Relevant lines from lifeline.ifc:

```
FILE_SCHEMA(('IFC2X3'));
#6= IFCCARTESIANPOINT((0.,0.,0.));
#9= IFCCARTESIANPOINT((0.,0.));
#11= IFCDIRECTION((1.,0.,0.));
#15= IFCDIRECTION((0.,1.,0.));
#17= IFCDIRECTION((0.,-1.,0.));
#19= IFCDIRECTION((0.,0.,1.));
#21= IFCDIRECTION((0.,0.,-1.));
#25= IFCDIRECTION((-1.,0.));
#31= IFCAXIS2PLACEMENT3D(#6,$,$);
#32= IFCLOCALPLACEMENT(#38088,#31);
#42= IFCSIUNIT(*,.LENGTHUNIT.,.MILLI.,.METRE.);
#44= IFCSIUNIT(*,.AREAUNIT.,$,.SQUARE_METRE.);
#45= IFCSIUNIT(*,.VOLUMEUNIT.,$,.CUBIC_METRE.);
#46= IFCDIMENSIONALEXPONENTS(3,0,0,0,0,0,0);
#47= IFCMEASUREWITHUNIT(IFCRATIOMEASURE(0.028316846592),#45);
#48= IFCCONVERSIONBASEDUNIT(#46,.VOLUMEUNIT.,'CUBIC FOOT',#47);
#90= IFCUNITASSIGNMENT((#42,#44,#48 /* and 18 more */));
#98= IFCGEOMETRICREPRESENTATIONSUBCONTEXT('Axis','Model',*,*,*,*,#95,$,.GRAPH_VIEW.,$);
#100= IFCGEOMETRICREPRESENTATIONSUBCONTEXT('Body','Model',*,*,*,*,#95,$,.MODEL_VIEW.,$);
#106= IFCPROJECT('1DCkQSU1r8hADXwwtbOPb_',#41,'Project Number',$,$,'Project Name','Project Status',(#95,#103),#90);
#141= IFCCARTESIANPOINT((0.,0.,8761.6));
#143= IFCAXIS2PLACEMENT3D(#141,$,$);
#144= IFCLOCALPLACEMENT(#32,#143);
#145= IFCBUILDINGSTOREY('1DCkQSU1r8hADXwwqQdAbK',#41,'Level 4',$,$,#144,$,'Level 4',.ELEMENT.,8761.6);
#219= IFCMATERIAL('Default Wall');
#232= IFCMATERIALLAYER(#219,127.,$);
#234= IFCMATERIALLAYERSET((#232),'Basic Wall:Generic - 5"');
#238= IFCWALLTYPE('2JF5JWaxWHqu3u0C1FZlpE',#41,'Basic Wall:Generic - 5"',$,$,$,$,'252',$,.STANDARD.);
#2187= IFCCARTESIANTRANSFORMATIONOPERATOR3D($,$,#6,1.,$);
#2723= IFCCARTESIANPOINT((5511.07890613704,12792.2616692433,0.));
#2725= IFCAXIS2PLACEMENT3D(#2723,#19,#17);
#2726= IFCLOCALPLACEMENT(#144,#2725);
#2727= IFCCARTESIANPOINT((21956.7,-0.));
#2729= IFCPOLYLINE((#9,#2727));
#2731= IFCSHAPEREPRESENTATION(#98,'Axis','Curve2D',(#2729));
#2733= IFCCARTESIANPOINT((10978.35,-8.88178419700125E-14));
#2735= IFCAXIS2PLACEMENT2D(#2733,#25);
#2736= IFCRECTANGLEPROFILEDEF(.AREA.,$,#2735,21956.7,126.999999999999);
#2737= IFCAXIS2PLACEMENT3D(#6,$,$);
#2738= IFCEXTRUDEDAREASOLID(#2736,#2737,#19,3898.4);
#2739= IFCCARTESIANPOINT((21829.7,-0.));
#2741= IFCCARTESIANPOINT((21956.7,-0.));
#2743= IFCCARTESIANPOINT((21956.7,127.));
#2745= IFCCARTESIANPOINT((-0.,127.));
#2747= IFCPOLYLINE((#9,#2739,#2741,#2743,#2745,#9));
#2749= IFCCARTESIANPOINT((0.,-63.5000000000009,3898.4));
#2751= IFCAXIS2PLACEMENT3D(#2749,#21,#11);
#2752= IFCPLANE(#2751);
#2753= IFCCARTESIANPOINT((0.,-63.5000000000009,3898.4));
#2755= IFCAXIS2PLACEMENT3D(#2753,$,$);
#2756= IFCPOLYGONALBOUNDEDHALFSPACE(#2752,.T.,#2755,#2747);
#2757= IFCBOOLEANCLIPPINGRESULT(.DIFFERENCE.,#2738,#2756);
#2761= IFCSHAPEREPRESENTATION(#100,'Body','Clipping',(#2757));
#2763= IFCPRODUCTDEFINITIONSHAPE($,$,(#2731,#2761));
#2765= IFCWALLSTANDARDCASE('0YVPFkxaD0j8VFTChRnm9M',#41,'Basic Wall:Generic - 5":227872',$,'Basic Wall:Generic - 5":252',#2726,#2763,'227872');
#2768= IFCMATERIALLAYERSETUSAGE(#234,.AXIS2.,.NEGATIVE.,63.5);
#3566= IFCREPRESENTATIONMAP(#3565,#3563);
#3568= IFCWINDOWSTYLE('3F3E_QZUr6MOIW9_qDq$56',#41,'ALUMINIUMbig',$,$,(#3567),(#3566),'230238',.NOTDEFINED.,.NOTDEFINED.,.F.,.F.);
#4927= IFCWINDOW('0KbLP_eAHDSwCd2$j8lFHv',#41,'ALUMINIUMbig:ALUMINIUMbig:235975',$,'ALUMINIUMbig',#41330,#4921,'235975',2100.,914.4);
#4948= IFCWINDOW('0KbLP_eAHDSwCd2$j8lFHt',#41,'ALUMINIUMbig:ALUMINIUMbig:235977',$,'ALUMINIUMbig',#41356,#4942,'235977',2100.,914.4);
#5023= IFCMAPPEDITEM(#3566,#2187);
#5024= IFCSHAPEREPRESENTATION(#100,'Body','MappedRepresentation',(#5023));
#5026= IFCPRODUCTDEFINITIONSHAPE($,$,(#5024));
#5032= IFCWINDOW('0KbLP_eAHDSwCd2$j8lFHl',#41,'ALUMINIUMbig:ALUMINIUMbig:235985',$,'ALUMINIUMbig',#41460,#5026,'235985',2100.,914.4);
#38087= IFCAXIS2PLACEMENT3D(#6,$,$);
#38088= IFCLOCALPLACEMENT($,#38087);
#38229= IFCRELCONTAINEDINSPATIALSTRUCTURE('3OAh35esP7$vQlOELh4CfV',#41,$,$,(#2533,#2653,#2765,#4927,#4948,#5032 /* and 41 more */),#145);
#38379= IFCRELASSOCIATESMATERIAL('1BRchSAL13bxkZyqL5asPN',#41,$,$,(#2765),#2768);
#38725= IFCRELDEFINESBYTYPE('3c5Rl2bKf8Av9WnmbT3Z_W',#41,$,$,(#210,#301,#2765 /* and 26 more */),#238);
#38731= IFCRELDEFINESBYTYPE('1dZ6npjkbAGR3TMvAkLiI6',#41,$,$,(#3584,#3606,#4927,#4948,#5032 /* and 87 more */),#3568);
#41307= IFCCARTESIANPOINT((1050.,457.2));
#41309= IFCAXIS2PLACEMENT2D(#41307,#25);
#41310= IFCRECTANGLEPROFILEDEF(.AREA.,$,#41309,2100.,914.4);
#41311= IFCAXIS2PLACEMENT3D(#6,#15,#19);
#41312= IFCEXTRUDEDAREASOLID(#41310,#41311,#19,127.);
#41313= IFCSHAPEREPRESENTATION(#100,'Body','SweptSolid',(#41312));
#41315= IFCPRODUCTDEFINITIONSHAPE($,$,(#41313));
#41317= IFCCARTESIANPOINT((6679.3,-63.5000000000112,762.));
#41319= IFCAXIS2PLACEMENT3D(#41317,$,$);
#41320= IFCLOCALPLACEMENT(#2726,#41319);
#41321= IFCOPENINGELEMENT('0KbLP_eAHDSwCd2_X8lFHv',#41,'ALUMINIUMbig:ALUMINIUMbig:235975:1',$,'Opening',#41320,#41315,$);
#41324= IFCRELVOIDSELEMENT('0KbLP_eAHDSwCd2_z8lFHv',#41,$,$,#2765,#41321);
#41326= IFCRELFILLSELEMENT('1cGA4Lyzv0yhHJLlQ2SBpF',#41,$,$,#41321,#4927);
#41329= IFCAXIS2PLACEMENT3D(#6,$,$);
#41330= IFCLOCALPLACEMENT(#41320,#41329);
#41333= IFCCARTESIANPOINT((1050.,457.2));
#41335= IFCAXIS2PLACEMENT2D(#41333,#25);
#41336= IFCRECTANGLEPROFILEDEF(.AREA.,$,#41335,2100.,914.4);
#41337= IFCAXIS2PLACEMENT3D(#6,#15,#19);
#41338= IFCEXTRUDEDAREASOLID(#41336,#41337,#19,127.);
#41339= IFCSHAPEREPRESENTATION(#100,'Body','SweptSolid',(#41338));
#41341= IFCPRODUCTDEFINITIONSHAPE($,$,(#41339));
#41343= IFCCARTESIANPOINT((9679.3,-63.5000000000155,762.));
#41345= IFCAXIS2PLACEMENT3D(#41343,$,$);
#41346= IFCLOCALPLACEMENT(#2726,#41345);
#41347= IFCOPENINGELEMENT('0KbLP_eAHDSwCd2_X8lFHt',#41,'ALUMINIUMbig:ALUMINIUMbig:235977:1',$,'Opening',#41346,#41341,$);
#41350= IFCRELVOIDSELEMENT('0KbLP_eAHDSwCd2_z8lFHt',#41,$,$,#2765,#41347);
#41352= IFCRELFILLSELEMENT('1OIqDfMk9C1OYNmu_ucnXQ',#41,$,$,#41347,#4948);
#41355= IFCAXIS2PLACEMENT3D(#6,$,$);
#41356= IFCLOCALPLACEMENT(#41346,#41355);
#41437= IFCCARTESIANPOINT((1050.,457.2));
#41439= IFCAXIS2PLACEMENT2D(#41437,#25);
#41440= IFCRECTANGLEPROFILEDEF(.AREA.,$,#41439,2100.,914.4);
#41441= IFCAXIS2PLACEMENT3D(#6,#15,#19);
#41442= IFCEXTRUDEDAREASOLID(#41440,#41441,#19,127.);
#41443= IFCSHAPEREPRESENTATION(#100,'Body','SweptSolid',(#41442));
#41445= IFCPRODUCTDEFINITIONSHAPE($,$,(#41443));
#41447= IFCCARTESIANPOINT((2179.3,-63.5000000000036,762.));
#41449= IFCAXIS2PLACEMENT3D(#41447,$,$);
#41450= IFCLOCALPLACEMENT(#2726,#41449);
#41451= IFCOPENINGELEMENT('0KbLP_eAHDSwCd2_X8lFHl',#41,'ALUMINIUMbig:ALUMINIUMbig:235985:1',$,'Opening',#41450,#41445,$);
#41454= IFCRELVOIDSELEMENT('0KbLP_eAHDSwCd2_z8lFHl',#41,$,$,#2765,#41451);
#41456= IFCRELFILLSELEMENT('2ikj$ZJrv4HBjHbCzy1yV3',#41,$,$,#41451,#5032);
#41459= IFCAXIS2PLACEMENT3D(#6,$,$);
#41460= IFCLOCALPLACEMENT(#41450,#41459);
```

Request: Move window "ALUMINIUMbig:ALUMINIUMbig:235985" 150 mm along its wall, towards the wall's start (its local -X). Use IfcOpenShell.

```python
import ifcopenshell
import ifcopenshell.api.geometry
import ifcopenshell.util.placement
import ifcopenshell.util.unit

model = ifcopenshell.open("lifeline.ifc")
unit_scale = ifcopenshell.util.unit.calculate_unit_scale(model)

window = model.by_guid("0KbLP_eAHDSwCd2$j8lFHl")
opening = window.FillsVoids[0].RelatingOpeningElement
wall = opening.VoidsElements[0].RelatingBuildingElement

wall_matrix = ifcopenshell.util.placement.get_local_placement(wall.ObjectPlacement)
shift = wall_matrix[:3, 0] * -0.15 / unit_scale
before = ifcopenshell.util.placement.get_local_placement(window.ObjectPlacement)[:3, 3].copy()

# The window is placed relative to its opening, so it follows when the opening moves.
matrix = ifcopenshell.util.placement.get_local_placement(opening.ObjectPlacement)
matrix[:3, 3] += shift
ifcopenshell.api.geometry.edit_object_placement(
    model, product=opening, matrix=matrix, is_si=False, should_transform_children=True
)

after = ifcopenshell.util.placement.get_local_placement(window.ObjectPlacement)[:3, 3]
print("window moved by", (after - before).round(3) + 0.0)

model.write("lifeline_updated.ifc")
```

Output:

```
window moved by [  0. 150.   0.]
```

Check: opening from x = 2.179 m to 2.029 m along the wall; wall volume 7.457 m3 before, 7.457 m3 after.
